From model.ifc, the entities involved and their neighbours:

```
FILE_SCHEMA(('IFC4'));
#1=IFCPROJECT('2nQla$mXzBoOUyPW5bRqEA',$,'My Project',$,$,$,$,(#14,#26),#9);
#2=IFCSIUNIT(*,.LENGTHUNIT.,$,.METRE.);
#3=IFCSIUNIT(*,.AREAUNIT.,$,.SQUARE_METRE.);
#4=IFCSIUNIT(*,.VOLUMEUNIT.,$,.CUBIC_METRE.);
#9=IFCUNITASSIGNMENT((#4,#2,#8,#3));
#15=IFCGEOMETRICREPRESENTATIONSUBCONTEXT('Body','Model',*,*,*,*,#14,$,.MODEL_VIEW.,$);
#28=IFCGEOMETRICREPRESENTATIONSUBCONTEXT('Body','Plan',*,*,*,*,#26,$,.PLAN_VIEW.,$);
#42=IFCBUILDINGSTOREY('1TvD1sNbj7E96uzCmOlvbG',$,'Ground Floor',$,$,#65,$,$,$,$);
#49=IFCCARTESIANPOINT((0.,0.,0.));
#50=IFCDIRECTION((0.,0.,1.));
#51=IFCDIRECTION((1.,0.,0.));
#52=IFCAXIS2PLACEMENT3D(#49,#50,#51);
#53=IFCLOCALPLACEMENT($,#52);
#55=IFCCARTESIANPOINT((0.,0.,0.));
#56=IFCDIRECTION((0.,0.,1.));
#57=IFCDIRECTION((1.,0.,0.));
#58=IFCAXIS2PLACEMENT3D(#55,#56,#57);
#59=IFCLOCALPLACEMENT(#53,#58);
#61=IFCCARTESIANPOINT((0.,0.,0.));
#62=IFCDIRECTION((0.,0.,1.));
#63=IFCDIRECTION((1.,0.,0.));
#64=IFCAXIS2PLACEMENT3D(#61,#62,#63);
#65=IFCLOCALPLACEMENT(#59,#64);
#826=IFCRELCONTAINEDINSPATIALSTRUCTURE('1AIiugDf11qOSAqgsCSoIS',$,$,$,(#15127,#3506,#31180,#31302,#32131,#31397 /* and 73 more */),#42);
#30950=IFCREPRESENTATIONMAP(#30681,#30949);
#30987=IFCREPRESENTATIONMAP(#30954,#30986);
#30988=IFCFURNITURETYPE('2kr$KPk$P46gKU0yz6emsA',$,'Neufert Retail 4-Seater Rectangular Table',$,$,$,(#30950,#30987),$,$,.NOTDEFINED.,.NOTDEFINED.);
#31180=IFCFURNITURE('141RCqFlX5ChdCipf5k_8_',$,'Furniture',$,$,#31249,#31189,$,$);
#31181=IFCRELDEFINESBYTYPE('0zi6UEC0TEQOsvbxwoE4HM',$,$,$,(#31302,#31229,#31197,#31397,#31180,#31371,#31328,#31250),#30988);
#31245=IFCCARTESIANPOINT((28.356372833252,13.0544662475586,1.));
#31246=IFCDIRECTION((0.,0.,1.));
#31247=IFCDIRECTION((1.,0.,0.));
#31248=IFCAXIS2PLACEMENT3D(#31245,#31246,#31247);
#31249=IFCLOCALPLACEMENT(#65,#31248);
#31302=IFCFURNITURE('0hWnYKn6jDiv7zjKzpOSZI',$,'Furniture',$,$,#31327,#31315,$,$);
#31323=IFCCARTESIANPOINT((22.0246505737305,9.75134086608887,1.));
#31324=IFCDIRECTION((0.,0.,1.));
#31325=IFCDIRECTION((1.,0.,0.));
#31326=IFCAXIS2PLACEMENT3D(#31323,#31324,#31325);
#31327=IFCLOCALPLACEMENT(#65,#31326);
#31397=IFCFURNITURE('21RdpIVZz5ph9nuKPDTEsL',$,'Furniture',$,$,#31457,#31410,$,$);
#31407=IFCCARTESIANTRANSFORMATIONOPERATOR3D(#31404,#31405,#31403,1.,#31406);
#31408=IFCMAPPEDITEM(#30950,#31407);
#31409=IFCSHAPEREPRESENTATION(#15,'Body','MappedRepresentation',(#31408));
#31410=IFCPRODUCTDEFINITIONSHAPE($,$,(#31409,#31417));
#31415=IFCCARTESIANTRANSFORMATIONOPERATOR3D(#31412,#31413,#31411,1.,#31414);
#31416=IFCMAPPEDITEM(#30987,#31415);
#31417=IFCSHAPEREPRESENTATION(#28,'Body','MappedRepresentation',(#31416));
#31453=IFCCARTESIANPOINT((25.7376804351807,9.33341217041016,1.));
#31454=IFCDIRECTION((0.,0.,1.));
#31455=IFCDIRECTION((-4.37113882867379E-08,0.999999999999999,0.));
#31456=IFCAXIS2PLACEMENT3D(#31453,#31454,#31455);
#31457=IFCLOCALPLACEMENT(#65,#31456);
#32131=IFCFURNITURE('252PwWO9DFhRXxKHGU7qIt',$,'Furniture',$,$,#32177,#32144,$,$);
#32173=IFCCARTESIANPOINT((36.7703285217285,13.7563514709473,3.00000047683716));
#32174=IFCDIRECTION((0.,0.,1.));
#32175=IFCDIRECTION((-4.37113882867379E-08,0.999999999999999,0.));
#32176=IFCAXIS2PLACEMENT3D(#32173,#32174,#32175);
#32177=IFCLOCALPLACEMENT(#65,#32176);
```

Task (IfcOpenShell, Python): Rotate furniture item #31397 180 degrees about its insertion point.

```python
import ifcopenshell
import ifcopenshell.api.geometry
import ifcopenshell.util.placement

model = ifcopenshell.open("model.ifc")

item = model.by_guid("21RdpIVZz5ph9nuKPDTEsL")
matrix = ifcopenshell.util.placement.get_local_placement(item.ObjectPlacement)
matrix = matrix @ ifcopenshell.util.placement.rotation(180, "Z")
ifcopenshell.api.geometry.edit_object_placement(model, product=item, matrix=matrix, is_si=False)

print(ifcopenshell.util.placement.get_local_placement(item.ObjectPlacement).round(3) + 0.0)

model.write("model_v2.ifc")
```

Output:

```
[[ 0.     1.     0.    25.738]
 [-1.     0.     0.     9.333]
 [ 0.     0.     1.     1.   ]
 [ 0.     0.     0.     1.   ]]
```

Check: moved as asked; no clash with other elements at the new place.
